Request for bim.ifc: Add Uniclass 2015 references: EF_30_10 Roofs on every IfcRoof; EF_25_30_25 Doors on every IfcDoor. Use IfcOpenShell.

First a look at what the model holds.

```python
import ifcopenshell

model = ifcopenshell.open("bim.ifc")
print(model.schema)
print("classifications:", [c.Name for c in model.by_type("IfcClassification")])
for ifc_class in ("IfcDoor", "IfcRoof", "IfcStair", "IfcWall", "IfcWindow"):
    print(ifc_class, len(model.by_type(ifc_class)))
```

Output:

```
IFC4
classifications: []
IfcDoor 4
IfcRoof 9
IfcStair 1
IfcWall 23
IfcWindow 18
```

```python
import ifcopenshell
import ifcopenshell.api.classification

model = ifcopenshell.open("bim.ifc")

system = ifcopenshell.api.classification.add_classification(model, classification="Uniclass 2015")

codes = {
    "IfcRoof": ("EF_30_10", "Roofs"),
    "IfcDoor": ("EF_25_30_25", "Doors"),
}
for ifc_class, (code, name) in codes.items():
    products = model.by_type(ifc_class)
    ifcopenshell.api.classification.add_reference(
        model, products=products, classification=system, identification=code, name=name
    )
    print(code, len(products))

model.write("bim-out.ifc")
```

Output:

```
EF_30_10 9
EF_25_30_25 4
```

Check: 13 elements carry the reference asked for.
